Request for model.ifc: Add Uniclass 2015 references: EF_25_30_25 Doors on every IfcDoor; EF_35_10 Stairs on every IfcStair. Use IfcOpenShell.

First a look at what the model holds.

```python
import ifcopenshell

model = ifcopenshell.open("model.ifc")
print(model.schema)
print("classifications:", [c.Name for c in model.by_type("IfcClassification")])
for ifc_class in ("IfcDoor", "IfcRoof", "IfcStair", "IfcWall", "IfcWindow"):
    print(ifc_class, len(model.by_type(ifc_class)))
```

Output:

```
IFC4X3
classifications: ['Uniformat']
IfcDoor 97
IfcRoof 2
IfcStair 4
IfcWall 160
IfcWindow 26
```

```python
import ifcopenshell
import ifcopenshell.api.classification

model = ifcopenshell.open("model.ifc")

system = ifcopenshell.api.classification.add_classification(model, classification="Uniclass 2015")

codes = {
    "IfcDoor": ("EF_25_30_25", "Doors"),
    "IfcStair": ("EF_35_10", "Stairs"),
}
for ifc_class, (code, name) in codes.items():
    products = model.by_type(ifc_class)
    ifcopenshell.api.classification.add_reference(
        model, products=products, classification=system, identification=code, name=name
    )
    print(code, len(products))

model.write("model-out.ifc")
```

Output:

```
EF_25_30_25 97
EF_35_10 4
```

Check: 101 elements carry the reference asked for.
